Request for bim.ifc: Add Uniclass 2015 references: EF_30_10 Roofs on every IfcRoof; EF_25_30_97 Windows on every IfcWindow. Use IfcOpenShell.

First a look at what the model holds.

```python
import ifcopenshell

model = ifcopenshell.open("bim.ifc")
print(model.schema)
print("classifications:", [c.Name for c in model.by_type("IfcClassification")])
for ifc_class in ("IfcDoor", "IfcRoof", "IfcStair", "IfcWall", "IfcWindow"):
    print(ifc_class, len(model.by_type(ifc_class)))
```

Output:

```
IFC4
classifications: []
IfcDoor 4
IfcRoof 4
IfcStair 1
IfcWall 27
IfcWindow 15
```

```python
import ifcopenshell
import ifcopenshell.api.classification

model = ifcopenshell.open("bim.ifc")

system = ifcopenshell.api.classification.add_classification(model, classification="Uniclass 2015")

codes = {
    "IfcRoof": ("EF_30_10", "Roofs"),
    "IfcWindow": ("EF_25_30_97", "Windows"),
}
for ifc_class, (code, name) in codes.items():
    products = model.by_type(ifc_class)
    ifcopenshell.api.classification.add_reference(
        model, products=products, classification=system, identification=code, name=name
    )
    print(code, len(products))

model.write("bim_rev.ifc")
```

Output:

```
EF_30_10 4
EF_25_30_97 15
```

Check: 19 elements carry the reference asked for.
